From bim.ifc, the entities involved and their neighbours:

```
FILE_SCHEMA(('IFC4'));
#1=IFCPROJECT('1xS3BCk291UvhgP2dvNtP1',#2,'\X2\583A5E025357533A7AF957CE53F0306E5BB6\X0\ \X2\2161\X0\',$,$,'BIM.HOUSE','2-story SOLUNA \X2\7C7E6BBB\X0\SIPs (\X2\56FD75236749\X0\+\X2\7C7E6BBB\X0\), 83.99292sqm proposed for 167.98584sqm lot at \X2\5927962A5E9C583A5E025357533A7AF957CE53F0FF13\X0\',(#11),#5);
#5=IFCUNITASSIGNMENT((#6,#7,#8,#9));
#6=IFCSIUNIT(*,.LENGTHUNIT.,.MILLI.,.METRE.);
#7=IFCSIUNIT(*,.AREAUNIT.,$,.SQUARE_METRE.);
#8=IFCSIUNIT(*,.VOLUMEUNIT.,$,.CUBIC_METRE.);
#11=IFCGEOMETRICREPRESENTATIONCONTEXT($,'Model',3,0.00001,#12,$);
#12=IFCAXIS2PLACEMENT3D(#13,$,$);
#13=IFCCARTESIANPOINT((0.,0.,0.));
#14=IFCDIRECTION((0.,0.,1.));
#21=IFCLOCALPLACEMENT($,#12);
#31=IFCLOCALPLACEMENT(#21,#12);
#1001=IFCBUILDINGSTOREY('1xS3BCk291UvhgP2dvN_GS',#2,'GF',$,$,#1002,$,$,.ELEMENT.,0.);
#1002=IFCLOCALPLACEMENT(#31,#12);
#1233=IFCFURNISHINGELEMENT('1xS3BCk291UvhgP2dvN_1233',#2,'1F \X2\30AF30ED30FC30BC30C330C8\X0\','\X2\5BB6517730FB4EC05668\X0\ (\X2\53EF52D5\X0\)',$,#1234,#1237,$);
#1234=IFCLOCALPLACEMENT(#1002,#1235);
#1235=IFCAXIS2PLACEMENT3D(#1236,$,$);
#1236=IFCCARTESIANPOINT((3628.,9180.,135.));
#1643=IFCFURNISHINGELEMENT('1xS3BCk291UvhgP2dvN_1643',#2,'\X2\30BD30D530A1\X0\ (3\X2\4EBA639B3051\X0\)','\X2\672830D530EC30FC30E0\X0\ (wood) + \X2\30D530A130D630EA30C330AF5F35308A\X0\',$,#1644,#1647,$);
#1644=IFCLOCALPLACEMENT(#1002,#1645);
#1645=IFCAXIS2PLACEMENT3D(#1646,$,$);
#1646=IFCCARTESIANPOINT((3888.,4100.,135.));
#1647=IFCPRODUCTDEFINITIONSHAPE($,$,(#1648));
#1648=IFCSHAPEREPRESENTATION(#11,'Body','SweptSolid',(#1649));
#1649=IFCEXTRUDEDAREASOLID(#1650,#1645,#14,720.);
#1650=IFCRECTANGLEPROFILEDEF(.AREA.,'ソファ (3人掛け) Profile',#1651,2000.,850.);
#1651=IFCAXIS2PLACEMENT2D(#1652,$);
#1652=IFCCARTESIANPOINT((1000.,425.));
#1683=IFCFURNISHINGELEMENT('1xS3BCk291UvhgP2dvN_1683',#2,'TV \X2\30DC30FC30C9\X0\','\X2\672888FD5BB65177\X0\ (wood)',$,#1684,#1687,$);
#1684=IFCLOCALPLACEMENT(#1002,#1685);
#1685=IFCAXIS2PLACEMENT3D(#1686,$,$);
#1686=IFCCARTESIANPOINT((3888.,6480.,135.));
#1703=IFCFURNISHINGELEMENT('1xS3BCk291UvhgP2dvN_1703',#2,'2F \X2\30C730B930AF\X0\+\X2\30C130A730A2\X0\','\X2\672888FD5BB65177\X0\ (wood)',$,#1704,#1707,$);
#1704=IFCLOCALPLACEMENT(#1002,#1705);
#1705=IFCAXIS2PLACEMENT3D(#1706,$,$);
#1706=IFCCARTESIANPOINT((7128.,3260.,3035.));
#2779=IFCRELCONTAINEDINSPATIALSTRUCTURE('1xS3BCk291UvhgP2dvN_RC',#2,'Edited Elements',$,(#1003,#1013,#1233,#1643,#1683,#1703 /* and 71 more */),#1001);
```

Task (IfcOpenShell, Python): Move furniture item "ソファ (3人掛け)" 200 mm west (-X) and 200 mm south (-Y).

```python
import ifcopenshell
import ifcopenshell.api.geometry
import ifcopenshell.util.placement
import ifcopenshell.util.unit

model = ifcopenshell.open("bim.ifc")
unit_scale = ifcopenshell.util.unit.calculate_unit_scale(model)

item = model.by_guid("1xS3BCk291UvhgP2dvN_1643")
matrix = ifcopenshell.util.placement.get_local_placement(item.ObjectPlacement)
matrix[0, 3] -= 0.2 / unit_scale
matrix[1, 3] -= 0.2 / unit_scale
ifcopenshell.api.geometry.edit_object_placement(model, product=item, matrix=matrix, is_si=False)

print(ifcopenshell.util.placement.get_local_placement(item.ObjectPlacement).round(3) + 0.0)

model.write("bim_rev.ifc")
```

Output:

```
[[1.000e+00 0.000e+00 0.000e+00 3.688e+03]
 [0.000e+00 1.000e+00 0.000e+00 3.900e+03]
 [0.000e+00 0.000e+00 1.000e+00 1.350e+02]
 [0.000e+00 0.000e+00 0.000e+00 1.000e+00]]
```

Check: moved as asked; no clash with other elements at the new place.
